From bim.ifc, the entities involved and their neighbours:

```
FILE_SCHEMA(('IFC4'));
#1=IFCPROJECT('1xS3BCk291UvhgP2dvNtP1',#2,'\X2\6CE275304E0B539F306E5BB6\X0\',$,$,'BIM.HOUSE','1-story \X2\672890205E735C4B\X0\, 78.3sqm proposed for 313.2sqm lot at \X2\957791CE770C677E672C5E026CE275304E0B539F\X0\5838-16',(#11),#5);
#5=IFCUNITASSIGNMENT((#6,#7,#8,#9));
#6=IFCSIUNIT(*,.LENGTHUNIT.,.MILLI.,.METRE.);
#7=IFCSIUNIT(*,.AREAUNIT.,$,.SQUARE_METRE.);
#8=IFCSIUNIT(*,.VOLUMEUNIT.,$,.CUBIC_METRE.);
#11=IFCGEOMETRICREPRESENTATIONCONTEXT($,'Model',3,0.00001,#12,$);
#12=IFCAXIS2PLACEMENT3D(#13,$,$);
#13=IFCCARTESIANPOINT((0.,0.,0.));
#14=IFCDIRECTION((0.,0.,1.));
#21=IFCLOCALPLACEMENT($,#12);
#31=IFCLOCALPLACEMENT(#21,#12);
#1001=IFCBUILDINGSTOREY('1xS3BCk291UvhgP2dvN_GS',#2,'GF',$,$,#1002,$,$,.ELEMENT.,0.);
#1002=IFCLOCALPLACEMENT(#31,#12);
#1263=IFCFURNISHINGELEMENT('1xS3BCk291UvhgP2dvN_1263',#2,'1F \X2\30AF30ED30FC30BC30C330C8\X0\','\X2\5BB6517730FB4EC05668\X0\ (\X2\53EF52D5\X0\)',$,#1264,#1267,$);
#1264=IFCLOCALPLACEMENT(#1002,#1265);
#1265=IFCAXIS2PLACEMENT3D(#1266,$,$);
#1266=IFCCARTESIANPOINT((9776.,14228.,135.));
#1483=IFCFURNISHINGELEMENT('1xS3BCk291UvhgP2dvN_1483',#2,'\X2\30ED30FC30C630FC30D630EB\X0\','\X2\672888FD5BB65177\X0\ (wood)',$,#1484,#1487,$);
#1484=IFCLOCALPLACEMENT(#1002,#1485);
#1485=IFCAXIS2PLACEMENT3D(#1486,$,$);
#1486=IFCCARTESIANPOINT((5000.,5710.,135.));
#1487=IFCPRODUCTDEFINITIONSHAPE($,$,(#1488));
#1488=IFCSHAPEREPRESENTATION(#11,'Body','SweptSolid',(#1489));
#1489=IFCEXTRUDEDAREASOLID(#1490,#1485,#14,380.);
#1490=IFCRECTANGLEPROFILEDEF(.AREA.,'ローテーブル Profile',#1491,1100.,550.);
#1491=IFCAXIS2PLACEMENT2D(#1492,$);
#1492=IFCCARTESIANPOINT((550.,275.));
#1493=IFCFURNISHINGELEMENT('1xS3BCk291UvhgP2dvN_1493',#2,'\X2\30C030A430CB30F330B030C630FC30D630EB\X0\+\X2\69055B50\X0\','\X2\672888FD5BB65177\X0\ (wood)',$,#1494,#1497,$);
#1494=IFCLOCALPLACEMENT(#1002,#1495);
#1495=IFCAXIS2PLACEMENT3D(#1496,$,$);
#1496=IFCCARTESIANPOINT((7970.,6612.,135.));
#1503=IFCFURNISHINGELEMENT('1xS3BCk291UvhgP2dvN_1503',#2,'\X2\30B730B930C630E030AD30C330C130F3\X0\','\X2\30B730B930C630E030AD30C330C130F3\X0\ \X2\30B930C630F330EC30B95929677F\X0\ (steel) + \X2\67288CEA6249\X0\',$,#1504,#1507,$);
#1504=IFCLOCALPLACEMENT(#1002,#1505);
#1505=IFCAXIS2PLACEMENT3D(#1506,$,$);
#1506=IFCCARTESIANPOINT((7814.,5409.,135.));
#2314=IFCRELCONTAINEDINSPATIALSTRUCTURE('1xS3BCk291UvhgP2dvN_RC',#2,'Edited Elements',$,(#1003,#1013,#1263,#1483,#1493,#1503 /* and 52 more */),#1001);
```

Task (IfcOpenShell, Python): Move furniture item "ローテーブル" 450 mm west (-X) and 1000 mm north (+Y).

```python
import ifcopenshell
import ifcopenshell.api.geometry
import ifcopenshell.util.placement
import ifcopenshell.util.unit

model = ifcopenshell.open("bim.ifc")
unit_scale = ifcopenshell.util.unit.calculate_unit_scale(model)

item = model.by_guid("1xS3BCk291UvhgP2dvN_1483")
matrix = ifcopenshell.util.placement.get_local_placement(item.ObjectPlacement)
matrix[0, 3] -= 0.45 / unit_scale
matrix[1, 3] += 1 / unit_scale
ifcopenshell.api.geometry.edit_object_placement(model, product=item, matrix=matrix, is_si=False)

print(ifcopenshell.util.placement.get_local_placement(item.ObjectPlacement).round(3) + 0.0)

model.write("bim_edited.ifc")
```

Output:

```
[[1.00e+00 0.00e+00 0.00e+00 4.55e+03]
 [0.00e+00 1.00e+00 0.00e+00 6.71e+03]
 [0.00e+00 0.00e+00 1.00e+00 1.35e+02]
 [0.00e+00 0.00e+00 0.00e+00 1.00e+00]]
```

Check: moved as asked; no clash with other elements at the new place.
